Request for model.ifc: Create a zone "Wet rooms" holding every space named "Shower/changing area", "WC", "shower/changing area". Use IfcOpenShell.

First a look at what the model holds.

```python
import ifcopenshell

model = ifcopenshell.open("model.ifc")
print(model.schema)
seen = {}
for space in model.by_type("IfcSpace"):
    seen[space.LongName] = seen.get(space.LongName, 0) + 1
for name, count in sorted(seen.items(), key=str):
    print(count, "x", name)
print("zones:", [z.Name for z in model.by_type("IfcZone")][:20])
```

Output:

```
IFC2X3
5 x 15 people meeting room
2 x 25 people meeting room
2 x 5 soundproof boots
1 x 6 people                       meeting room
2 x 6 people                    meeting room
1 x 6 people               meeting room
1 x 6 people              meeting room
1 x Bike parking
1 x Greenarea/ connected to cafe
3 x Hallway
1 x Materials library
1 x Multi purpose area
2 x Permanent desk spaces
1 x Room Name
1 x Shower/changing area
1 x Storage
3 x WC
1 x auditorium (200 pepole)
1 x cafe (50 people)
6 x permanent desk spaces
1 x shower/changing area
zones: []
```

```python
import ifcopenshell
import ifcopenshell.api.group
import ifcopenshell.api.root

model = ifcopenshell.open("model.ifc")

names = {"Shower/changing area", "WC", "shower/changing area"}
spaces = [s for s in model.by_type("IfcSpace") if s.LongName in names]

zone = ifcopenshell.api.root.create_entity(model, ifc_class="IfcZone", name="Wet rooms")
ifcopenshell.api.group.assign_group(model, products=spaces, group=zone)
print(len(spaces), "spaces in", zone.Name)

model.write("model_edited.ifc")
```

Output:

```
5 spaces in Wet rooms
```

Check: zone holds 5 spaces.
